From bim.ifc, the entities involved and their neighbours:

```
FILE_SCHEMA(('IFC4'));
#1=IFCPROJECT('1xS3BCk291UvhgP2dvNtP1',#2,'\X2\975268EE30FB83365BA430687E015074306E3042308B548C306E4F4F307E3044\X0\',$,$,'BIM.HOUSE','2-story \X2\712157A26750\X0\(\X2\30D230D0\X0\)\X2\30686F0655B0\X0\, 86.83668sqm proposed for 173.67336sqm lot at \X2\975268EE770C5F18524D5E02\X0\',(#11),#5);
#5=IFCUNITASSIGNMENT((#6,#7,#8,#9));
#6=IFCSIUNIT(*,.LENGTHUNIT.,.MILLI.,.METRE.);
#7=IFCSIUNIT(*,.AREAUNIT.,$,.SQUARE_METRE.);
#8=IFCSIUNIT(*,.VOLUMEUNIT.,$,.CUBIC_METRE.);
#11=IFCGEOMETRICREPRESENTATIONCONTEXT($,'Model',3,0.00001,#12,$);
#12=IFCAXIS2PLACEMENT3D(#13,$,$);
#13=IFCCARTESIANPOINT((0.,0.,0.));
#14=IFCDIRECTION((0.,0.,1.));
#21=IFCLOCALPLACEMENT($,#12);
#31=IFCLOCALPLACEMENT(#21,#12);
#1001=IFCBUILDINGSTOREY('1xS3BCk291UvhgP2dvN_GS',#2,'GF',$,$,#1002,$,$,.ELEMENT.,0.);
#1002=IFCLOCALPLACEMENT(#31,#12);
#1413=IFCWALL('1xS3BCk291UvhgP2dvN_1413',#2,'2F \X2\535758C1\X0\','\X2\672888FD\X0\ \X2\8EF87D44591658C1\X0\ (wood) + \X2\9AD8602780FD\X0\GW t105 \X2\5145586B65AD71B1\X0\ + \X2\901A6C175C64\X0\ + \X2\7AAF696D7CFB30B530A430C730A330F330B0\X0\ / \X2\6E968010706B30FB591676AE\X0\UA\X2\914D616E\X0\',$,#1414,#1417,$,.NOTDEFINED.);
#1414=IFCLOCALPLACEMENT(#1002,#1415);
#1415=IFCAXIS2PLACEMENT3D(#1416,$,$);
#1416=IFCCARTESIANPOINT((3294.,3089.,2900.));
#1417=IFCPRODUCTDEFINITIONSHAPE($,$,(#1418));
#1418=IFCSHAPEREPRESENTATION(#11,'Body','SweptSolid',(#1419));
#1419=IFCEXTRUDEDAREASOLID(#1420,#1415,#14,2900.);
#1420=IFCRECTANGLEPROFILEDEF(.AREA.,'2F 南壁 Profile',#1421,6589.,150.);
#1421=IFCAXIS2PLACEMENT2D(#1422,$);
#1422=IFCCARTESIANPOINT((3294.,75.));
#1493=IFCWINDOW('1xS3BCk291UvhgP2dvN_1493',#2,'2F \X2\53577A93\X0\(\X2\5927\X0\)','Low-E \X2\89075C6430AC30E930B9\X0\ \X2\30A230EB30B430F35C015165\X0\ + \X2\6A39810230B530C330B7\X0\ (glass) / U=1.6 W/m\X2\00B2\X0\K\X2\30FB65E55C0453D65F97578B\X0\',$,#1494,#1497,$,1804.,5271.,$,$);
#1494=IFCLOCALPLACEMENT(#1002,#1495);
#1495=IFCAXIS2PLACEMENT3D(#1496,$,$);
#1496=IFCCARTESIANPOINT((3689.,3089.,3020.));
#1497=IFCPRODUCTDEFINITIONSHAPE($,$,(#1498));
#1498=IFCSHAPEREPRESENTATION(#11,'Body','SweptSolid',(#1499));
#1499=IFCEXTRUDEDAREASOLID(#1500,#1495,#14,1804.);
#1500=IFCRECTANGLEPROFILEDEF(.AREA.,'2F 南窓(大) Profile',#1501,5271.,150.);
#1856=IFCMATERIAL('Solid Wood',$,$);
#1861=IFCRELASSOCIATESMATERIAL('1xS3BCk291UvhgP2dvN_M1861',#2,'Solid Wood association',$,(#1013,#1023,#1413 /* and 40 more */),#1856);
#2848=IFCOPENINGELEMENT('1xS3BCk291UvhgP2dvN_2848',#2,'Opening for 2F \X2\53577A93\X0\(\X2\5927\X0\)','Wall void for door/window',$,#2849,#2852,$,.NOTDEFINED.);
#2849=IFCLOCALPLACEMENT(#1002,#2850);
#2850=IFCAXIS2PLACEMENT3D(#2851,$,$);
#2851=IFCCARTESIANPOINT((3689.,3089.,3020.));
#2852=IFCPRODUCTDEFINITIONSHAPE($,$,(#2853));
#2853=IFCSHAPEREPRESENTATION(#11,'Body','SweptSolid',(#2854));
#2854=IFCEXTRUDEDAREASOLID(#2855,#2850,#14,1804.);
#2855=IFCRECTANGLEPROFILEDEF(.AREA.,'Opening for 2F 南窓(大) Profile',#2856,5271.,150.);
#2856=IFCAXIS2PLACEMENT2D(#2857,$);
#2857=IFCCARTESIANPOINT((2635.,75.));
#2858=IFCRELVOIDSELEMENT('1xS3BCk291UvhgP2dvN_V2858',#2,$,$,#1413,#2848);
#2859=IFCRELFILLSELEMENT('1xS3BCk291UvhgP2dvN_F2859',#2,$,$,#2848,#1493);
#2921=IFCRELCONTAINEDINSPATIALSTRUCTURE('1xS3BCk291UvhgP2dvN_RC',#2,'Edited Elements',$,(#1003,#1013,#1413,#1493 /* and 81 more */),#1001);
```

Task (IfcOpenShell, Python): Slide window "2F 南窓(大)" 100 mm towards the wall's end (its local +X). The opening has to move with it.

```python
import ifcopenshell
import ifcopenshell.api.geometry
import ifcopenshell.util.placement

model = ifcopenshell.open("bim.ifc")

window = model.by_guid("1xS3BCk291UvhgP2dvN_1493")
opening = window.FillsVoids[0].RelatingOpeningElement
wall = opening.VoidsElements[0].RelatingBuildingElement

wall_matrix = ifcopenshell.util.placement.get_local_placement(wall.ObjectPlacement)
shift = wall_matrix[:3, 0] * 100.0
before = ifcopenshell.util.placement.get_local_placement(window.ObjectPlacement)[:3, 3].copy()

# The window is not placed relative to its opening, so move both.
for product in (opening, window):
    matrix = ifcopenshell.util.placement.get_local_placement(product.ObjectPlacement)
    matrix[:3, 3] += shift
    ifcopenshell.api.geometry.edit_object_placement(model, product=product, matrix=matrix, is_si=False)

after = ifcopenshell.util.placement.get_local_placement(window.ObjectPlacement)[:3, 3]
print("window moved by", (after - before).round(3) + 0.0)

model.write("bim_edited.ifc")
```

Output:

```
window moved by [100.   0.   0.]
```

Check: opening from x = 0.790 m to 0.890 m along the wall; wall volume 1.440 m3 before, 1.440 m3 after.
